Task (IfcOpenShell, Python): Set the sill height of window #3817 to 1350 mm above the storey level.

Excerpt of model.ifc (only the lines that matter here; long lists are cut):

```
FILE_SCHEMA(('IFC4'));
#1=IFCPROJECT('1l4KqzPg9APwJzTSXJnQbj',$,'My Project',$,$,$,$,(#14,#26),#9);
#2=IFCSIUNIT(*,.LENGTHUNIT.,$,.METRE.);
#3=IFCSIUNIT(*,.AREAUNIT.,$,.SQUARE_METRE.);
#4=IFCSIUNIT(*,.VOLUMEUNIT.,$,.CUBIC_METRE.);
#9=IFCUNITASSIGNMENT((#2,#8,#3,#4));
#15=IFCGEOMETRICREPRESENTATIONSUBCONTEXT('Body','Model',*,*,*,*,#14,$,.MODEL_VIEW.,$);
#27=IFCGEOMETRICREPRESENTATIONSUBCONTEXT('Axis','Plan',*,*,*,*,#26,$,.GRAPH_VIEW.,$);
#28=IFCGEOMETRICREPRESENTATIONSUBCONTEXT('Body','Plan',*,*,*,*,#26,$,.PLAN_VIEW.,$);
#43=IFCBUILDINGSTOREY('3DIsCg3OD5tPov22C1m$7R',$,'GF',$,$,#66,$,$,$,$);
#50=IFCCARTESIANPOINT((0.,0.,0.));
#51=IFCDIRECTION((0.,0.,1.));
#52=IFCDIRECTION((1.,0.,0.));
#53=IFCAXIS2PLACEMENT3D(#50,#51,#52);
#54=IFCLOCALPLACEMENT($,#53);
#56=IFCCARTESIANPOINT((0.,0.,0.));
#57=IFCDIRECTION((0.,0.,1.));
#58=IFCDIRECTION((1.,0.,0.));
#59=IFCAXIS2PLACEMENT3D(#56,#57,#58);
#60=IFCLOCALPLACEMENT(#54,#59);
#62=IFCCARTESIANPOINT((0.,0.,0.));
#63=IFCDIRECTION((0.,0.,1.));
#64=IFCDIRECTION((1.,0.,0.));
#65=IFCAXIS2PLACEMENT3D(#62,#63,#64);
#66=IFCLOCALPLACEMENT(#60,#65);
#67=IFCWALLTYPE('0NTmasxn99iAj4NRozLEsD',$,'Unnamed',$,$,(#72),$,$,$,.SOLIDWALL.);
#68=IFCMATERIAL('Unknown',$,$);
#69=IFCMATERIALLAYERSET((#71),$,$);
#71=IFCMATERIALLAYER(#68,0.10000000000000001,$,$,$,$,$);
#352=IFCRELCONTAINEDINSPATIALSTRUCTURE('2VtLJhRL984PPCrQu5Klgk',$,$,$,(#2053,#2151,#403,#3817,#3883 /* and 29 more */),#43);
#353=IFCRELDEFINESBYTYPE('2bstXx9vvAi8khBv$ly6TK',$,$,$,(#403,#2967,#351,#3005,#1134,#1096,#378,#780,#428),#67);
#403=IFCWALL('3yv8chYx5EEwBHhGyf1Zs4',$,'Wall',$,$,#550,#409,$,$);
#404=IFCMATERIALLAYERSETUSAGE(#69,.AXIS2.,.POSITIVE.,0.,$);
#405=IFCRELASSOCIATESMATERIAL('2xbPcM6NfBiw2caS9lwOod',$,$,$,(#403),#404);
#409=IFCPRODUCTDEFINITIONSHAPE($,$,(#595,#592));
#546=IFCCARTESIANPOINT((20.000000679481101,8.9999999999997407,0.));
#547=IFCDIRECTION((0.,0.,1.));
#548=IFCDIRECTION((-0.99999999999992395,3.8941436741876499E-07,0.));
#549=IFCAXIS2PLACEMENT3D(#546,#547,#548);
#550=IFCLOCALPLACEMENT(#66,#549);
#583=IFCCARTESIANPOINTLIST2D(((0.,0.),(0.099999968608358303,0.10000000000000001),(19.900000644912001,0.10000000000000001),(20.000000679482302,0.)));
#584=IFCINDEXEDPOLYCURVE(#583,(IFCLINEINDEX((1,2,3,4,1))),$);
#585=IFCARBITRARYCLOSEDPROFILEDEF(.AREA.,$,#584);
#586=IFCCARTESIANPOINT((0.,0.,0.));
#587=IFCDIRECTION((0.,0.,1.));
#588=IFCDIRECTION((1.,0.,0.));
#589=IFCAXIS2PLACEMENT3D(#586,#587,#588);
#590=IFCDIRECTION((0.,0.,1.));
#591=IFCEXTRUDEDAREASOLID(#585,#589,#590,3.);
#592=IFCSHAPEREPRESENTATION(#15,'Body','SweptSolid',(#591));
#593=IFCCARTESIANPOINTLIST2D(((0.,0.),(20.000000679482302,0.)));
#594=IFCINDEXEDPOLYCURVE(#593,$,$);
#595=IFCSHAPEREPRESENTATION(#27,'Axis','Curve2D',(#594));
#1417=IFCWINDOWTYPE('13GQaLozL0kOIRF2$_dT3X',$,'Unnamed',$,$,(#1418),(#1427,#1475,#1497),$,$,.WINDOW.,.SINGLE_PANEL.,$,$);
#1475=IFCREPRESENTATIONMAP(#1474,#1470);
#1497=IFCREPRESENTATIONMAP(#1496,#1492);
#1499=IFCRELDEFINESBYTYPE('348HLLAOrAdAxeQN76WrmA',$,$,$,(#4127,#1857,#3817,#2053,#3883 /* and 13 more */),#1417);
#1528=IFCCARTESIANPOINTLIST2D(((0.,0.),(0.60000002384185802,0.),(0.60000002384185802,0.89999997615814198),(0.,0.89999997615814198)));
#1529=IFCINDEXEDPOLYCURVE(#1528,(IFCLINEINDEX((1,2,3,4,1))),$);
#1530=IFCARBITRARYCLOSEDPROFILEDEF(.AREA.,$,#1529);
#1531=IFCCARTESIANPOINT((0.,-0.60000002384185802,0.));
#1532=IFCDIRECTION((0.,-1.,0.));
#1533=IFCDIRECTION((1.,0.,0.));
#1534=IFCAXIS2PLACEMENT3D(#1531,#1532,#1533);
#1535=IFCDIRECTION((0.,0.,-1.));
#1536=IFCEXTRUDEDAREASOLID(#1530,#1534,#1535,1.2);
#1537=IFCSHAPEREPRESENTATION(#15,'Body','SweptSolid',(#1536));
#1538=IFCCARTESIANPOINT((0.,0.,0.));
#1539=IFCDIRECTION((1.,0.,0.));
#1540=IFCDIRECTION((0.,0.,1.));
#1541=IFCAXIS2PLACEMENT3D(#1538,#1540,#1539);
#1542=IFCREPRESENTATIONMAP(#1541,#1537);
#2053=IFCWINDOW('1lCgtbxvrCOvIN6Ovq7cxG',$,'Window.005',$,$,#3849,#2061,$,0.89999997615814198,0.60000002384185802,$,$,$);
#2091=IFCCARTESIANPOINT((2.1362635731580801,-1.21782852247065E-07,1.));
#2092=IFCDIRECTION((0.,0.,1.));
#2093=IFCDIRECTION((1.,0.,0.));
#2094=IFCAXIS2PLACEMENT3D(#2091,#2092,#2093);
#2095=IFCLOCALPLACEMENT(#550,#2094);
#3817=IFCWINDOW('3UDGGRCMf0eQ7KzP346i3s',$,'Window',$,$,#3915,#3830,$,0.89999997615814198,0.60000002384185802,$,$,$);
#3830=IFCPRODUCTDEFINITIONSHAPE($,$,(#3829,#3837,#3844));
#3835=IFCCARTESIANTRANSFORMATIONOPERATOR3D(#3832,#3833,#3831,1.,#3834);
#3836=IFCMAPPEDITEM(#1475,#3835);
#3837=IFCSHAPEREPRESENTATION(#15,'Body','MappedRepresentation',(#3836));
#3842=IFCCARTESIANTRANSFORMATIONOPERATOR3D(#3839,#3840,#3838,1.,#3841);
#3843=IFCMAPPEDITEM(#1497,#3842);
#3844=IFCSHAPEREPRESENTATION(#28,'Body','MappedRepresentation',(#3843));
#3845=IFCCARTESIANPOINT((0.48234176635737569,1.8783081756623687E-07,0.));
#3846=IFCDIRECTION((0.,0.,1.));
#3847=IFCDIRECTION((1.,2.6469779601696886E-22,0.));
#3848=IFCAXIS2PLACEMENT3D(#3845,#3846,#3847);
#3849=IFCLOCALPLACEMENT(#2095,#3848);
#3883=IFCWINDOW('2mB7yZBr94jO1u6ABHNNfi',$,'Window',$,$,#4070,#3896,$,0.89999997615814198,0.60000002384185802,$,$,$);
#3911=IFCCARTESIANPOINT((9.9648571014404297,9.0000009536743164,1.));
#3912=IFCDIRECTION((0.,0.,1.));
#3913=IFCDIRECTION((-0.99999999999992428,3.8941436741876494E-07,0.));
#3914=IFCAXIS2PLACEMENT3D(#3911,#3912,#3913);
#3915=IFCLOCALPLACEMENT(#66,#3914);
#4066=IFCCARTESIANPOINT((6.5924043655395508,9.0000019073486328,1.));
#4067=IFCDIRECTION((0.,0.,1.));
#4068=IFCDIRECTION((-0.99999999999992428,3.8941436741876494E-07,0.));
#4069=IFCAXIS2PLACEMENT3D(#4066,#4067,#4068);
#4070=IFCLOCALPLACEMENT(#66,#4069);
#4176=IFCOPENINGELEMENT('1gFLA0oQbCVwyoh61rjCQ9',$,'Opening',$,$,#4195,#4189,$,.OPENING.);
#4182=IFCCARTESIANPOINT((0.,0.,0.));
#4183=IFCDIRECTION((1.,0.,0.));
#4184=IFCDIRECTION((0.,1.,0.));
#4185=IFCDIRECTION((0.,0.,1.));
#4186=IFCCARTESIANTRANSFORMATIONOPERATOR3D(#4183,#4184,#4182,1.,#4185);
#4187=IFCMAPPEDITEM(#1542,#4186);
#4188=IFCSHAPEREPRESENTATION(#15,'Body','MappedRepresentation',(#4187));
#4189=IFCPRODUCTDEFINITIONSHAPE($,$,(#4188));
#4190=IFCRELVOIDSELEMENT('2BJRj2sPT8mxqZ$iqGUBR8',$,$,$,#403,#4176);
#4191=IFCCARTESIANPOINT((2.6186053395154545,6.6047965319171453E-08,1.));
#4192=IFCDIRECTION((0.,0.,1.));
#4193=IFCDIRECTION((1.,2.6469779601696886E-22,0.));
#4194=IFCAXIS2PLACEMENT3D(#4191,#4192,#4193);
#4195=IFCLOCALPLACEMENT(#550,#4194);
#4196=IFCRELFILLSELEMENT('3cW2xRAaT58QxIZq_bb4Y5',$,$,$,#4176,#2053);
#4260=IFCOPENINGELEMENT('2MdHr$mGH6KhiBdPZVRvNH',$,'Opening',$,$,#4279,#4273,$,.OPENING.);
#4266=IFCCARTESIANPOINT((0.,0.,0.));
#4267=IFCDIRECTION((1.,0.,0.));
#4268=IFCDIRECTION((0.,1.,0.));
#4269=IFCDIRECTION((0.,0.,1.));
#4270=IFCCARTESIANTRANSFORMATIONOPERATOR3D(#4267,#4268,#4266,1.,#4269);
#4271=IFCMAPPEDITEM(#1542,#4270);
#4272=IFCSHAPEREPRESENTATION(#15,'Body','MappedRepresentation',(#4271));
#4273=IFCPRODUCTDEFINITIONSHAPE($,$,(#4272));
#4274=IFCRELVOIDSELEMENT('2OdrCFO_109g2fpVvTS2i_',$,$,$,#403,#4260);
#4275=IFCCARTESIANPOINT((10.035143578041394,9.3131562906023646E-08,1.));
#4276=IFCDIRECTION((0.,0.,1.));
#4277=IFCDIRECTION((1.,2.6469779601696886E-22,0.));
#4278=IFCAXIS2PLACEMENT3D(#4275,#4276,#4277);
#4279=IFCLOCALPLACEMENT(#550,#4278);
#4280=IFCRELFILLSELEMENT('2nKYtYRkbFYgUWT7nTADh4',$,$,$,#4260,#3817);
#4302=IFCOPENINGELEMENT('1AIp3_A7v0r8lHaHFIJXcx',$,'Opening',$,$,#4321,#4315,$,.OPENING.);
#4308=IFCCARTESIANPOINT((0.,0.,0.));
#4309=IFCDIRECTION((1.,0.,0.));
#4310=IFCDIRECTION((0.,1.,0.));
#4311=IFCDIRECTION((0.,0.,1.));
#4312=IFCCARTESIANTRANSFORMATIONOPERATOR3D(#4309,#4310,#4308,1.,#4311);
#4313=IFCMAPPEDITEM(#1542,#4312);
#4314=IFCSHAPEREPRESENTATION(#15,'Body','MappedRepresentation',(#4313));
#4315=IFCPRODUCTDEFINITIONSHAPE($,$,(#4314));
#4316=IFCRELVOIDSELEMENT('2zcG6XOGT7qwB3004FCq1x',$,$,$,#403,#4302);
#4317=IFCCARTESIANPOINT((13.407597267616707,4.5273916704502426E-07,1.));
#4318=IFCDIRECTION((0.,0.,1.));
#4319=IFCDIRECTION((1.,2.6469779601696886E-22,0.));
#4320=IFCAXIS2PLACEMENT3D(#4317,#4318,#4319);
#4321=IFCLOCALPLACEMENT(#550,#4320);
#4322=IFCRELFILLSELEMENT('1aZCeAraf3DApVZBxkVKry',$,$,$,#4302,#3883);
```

```python
import numpy as np
import ifcopenshell
import ifcopenshell.api.geometry
import ifcopenshell.geom
import ifcopenshell.util.element
import ifcopenshell.util.placement
import ifcopenshell.util.shape
import ifcopenshell.util.unit

model = ifcopenshell.open("model.ifc")
unit_scale = ifcopenshell.util.unit.calculate_unit_scale(model)

window = model.by_guid("3UDGGRCMf0eQ7KzP346i3s")
opening = window.FillsVoids[0].RelatingOpeningElement
storey = ifcopenshell.util.element.get_container(window, ifc_class="IfcBuildingStorey")
level = ifcopenshell.util.placement.get_local_placement(storey.ObjectPlacement)[2, 3]

# The opening's origin need not be at the sill, so measure its lowest point.
shape = ifcopenshell.geom.create_shape(ifcopenshell.geom.settings(), opening)
bottom = ifcopenshell.util.shape.get_shape_bottom_elevation(shape, shape.geometry) / unit_scale
dz = level + 1.35 / unit_scale - bottom

shift = np.array([0.0, 0.0, dz])
# The window is not placed relative to its opening, so move both.
for product in (opening, window):
    matrix = ifcopenshell.util.placement.get_local_placement(product.ObjectPlacement)
    matrix[:3, 3] += shift
    ifcopenshell.api.geometry.edit_object_placement(model, product=product, matrix=matrix, is_si=False)

print(f"moved by {dz * unit_scale:+.3f} m")

model.write("model_updated.ifc")
```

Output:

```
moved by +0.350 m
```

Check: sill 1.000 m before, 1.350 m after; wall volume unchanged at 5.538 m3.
